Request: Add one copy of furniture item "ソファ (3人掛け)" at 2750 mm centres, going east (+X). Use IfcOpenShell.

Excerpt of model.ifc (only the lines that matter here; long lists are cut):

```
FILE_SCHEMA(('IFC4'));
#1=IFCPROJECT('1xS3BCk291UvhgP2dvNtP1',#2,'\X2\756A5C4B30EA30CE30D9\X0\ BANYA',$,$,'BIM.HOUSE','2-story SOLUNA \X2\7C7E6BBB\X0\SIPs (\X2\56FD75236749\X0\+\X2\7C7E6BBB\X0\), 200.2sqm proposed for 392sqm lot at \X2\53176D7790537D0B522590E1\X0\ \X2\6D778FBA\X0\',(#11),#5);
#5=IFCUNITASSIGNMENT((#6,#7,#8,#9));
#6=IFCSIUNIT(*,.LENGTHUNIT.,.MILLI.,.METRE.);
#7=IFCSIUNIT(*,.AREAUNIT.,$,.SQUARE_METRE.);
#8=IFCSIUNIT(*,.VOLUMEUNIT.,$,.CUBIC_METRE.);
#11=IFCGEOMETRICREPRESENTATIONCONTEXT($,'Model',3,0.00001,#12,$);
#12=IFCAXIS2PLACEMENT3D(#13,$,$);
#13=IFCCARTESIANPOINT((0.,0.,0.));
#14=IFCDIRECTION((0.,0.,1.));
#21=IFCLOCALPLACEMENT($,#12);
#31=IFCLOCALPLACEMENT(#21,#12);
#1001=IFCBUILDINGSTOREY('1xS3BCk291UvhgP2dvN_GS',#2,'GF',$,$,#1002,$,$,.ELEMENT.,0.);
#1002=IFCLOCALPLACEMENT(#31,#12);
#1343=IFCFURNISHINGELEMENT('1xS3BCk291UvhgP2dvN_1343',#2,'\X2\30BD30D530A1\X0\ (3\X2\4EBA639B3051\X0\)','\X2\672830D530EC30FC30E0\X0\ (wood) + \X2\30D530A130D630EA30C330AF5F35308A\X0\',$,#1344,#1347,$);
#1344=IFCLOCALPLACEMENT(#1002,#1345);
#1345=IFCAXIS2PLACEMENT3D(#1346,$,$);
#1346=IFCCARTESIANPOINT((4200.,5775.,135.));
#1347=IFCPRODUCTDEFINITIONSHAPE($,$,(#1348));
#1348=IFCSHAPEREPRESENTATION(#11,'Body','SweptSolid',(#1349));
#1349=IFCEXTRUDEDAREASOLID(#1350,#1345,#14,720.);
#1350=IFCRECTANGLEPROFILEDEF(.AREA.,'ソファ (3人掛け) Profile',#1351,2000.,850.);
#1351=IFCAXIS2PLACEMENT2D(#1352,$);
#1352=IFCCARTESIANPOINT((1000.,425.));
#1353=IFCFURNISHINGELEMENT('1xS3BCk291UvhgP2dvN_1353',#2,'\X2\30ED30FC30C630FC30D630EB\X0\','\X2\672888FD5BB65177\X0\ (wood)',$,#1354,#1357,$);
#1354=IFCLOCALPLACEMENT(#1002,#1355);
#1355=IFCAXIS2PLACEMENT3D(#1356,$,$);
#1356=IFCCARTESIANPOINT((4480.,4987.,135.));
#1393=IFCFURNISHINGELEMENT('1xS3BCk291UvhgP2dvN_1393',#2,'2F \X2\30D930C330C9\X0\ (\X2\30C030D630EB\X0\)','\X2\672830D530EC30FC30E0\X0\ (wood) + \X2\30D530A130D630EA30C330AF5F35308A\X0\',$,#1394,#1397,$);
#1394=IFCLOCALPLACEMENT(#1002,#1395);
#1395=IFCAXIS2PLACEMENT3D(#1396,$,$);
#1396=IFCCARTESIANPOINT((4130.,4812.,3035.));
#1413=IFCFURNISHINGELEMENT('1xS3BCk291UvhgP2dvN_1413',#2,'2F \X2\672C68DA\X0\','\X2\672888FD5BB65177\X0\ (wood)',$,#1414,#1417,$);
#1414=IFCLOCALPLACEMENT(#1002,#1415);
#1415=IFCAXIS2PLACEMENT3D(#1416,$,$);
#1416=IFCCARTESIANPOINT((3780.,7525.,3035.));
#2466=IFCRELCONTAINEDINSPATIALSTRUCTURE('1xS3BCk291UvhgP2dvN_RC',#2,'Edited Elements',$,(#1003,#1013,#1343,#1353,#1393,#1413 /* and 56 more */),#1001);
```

```python
import numpy as np
import ifcopenshell
import ifcopenshell.api.geometry
import ifcopenshell.api.root
import ifcopenshell.util.element
import ifcopenshell.util.placement
import ifcopenshell.util.unit

model = ifcopenshell.open("model.ifc")
unit_scale = ifcopenshell.util.unit.calculate_unit_scale(model)


def reuse_history(source, copy):
    """copy_class also copies each property set's owner history, people and application; keep the originals."""
    for rel in copy.IsDefinedBy:
        if rel.is_a("IfcRelDefinesByProperties") and (history := rel.RelatingPropertyDefinition.OwnerHistory):
            rel.RelatingPropertyDefinition.OwnerHistory = source.OwnerHistory
            ifcopenshell.util.element.remove_deep2(model, history)


source = model.by_id(1343)
base = ifcopenshell.util.placement.get_local_placement(source.ObjectPlacement)
step = np.array([1.0, 0.0, 0.0]) * 2.75 / unit_scale

for i in range(1, 2):
    copy = ifcopenshell.api.root.copy_class(model, product=source)
    copy.Representation = ifcopenshell.util.element.copy_deep(
        model, source.Representation, exclude=["IfcGeometricRepresentationContext", "IfcRepresentationMap"]
    )
    reuse_history(source, copy)
    matrix = base.copy()
    matrix[:3, 3] += i * step
    print("added at", matrix[:3, 3].round(3) + 0.0)
    ifcopenshell.api.geometry.edit_object_placement(model, product=copy, matrix=matrix, is_si=False)

model.write("model_edited.ifc")
```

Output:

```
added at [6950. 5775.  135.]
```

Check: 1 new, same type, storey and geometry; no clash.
